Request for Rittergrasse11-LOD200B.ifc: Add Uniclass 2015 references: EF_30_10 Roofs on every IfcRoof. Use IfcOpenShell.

First a look at what the model holds.

```python
import ifcopenshell

model = ifcopenshell.open("Rittergrasse11-LOD200B.ifc")
print(model.schema)
print("classifications:", [c.Name for c in model.by_type("IfcClassification")])
for ifc_class in ("IfcDoor", "IfcRoof", "IfcStair", "IfcWall", "IfcWindow"):
    print(ifc_class, len(model.by_type(ifc_class)))
```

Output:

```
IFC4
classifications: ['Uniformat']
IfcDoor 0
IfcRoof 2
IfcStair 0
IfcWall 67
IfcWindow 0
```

```python
import ifcopenshell
import ifcopenshell.api.classification

model = ifcopenshell.open("Rittergrasse11-LOD200B.ifc")

system = ifcopenshell.api.classification.add_classification(model, classification="Uniclass 2015")

codes = {
    "IfcRoof": ("EF_30_10", "Roofs"),
}
for ifc_class, (code, name) in codes.items():
    products = model.by_type(ifc_class)
    ifcopenshell.api.classification.add_reference(
        model, products=products, classification=system, identification=code, name=name
    )
    print(code, len(products))

model.write("Rittergrasse11-LOD200B_edited.ifc")
```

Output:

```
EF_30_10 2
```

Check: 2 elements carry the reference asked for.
